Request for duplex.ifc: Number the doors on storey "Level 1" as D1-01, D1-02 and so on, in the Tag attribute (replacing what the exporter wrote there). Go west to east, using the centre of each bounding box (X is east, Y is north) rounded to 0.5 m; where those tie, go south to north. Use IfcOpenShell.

First a look at what the model holds.

```python
import ifcopenshell
import ifcopenshell.util.element
import ifcopenshell.util.placement

model = ifcopenshell.open("duplex.ifc")
print(model.schema)
storey = next(s for s in model.by_type("IfcBuildingStorey") if s.Name == "Level 1")
doors = [e for e in ifcopenshell.util.element.get_decomposition(storey) if e.is_a("IfcDoor")]
for e in sorted(doors, key=lambda e: e.id()):
    origin = ifcopenshell.util.placement.get_local_placement(e.ObjectPlacement)[:3, 3]
    print(e.id(), e.Tag, e.Name, origin.round(2) + 0.0, sep=" | ")
```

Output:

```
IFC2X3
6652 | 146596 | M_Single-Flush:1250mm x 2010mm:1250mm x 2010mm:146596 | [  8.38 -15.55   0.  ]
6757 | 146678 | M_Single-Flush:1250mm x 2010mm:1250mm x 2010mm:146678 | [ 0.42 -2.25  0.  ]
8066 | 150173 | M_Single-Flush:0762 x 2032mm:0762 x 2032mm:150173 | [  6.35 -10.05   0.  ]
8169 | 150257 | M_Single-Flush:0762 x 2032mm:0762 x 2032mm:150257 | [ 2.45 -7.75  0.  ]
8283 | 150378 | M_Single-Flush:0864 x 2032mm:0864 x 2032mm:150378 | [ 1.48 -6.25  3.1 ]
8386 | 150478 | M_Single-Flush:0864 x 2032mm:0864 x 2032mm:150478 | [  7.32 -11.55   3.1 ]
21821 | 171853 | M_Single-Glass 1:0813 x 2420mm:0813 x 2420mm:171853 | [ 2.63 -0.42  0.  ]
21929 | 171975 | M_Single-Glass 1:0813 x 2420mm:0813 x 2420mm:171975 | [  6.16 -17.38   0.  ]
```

```python
import ifcopenshell
import ifcopenshell.geom
import ifcopenshell.util.element
import ifcopenshell.util.shape

model = ifcopenshell.open("duplex.ifc")
settings = ifcopenshell.geom.settings()
settings.set("use-world-coords", True)


def centre(element):
    shape = ifcopenshell.geom.create_shape(settings, element)
    return ifcopenshell.util.shape.get_bbox_centroid(shape.geometry)


storey = next(s for s in model.by_type("IfcBuildingStorey") if s.Name == "Level 1")
doors = [e for e in ifcopenshell.util.element.get_decomposition(storey) if e.is_a("IfcDoor")]

# Insertion points can sit at a corner or the storey origin, so sort by the geometry (in metres).
centres = {e: centre(e) for e in doors}
doors.sort(key=lambda e: (round(centres[e][0] / 0.5), centres[e][1]))

for i, e in enumerate(doors, start=1):
    number = f"D1-{i:02d}"
    e.Tag = number
    print(e.id(), number)

model.write("duplex_rev.ifc")
```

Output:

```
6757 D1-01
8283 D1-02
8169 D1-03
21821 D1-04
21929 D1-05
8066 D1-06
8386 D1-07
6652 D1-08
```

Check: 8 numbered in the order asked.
